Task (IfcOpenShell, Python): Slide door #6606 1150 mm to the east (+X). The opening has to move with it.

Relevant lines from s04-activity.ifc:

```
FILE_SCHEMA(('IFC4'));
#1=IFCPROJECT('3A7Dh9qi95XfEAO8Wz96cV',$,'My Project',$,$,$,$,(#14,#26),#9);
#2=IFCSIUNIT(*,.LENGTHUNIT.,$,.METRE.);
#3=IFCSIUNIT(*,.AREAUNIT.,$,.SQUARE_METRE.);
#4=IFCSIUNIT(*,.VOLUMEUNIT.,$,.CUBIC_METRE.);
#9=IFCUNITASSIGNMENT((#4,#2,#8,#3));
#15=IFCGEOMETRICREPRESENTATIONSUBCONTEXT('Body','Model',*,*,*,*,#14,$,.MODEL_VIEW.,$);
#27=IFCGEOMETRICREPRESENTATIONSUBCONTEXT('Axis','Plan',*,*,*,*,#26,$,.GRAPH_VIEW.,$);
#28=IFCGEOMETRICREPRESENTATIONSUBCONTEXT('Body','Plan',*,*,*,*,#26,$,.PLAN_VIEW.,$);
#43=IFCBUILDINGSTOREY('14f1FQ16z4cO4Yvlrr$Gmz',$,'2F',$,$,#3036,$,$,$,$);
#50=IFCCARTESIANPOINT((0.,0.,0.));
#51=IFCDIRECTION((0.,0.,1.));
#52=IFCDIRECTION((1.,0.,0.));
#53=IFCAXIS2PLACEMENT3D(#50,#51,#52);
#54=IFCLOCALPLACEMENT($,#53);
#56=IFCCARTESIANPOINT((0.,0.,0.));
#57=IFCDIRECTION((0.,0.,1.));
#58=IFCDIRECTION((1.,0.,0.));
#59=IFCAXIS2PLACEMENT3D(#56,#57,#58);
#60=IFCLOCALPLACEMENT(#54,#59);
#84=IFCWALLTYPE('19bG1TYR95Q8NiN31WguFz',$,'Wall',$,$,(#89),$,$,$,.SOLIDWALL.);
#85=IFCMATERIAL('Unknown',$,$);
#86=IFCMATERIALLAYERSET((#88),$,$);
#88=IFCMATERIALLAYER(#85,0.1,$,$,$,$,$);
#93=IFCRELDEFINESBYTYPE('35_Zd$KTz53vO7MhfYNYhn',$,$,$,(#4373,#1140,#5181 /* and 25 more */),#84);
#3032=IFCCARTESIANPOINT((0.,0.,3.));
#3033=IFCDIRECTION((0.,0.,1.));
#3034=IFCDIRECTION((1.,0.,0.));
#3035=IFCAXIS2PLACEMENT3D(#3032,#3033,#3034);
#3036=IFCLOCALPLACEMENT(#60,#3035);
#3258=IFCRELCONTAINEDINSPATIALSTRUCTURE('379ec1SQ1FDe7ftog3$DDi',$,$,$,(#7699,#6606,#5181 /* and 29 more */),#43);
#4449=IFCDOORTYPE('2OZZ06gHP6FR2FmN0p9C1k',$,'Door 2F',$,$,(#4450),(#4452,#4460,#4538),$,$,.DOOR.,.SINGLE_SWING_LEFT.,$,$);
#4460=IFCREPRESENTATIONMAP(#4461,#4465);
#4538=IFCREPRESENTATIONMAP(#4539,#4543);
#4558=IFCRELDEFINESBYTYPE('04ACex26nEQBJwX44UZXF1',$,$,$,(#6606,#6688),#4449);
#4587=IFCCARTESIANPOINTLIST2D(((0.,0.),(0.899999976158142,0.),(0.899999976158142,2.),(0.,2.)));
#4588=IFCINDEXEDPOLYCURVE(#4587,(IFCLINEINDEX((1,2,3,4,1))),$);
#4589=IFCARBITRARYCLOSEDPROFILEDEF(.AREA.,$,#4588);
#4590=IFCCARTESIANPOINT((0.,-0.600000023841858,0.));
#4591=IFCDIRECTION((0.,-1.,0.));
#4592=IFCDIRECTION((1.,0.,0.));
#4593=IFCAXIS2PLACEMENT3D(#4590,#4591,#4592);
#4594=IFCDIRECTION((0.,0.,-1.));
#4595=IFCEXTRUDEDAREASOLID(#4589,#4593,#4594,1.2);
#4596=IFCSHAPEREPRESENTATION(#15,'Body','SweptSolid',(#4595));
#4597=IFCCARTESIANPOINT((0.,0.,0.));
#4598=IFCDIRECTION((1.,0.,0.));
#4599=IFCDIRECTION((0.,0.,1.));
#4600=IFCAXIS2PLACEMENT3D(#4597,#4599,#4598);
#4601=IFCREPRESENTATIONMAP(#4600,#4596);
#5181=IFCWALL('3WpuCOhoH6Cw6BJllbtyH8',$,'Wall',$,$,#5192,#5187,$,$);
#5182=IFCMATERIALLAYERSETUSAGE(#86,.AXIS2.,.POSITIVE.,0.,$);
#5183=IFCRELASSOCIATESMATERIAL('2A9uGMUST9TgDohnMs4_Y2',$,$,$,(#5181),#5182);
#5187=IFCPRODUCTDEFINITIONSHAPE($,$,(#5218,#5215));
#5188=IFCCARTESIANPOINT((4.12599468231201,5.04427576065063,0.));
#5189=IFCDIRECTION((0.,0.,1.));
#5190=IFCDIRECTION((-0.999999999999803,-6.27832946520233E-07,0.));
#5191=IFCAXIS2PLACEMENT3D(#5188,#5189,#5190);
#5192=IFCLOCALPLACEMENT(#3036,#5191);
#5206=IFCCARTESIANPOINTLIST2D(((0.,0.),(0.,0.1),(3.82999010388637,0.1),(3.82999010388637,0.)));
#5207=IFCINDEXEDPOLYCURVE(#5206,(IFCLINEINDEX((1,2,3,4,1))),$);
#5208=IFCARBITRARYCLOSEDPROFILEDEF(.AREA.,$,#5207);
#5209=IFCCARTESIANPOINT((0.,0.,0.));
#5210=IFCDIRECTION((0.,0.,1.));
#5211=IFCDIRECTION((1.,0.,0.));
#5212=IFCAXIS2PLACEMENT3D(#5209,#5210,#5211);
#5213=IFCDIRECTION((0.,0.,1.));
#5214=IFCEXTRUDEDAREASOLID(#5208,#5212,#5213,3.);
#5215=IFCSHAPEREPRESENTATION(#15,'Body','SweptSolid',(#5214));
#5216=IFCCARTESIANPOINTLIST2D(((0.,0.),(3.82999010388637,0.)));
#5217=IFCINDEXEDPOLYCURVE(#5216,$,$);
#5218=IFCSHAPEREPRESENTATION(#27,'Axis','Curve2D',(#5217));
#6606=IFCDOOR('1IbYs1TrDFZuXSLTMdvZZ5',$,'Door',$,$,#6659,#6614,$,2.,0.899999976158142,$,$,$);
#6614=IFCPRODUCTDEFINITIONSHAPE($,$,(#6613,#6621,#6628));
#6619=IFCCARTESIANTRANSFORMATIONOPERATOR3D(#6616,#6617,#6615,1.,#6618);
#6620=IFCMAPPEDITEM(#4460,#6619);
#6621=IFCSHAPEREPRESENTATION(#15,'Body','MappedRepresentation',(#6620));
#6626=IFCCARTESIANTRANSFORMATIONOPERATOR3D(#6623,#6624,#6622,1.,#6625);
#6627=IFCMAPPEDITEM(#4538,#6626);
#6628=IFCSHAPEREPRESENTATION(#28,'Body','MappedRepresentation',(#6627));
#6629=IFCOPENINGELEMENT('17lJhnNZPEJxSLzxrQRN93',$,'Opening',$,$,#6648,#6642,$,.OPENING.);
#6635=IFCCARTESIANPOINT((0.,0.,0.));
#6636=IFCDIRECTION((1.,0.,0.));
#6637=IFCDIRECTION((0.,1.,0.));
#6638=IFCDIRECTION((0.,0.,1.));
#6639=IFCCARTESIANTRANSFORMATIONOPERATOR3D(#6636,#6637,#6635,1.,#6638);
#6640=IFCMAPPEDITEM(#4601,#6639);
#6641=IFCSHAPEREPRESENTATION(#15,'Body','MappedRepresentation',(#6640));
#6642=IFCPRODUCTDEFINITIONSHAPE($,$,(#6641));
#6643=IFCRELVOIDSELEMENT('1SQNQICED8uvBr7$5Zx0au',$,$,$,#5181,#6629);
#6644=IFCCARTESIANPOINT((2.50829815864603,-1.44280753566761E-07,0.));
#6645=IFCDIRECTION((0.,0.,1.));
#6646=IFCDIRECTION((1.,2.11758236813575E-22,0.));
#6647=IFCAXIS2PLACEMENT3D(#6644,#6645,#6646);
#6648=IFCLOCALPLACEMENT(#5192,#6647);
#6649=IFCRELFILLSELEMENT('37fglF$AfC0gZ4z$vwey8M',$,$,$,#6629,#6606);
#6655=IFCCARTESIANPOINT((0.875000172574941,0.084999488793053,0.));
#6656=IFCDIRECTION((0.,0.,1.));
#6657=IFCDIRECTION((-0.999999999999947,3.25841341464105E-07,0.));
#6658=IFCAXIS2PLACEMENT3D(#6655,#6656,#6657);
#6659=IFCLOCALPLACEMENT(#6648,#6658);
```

```python
import ifcopenshell
import ifcopenshell.api.geometry
import ifcopenshell.util.placement
import ifcopenshell.util.unit

model = ifcopenshell.open("s04-activity.ifc")
unit_scale = ifcopenshell.util.unit.calculate_unit_scale(model)

door = model.by_id(6606)
opening = door.FillsVoids[0].RelatingOpeningElement
wall = opening.VoidsElements[0].RelatingBuildingElement

wall_matrix = ifcopenshell.util.placement.get_local_placement(wall.ObjectPlacement)
shift = wall_matrix[:3, 0] * -1.15 / unit_scale
before = ifcopenshell.util.placement.get_local_placement(door.ObjectPlacement)[:3, 3].copy()

# The door is placed relative to its opening, so it follows when the opening moves.
matrix = ifcopenshell.util.placement.get_local_placement(opening.ObjectPlacement)
matrix[:3, 3] += shift
ifcopenshell.api.geometry.edit_object_placement(
    model, product=opening, matrix=matrix, is_si=False, should_transform_children=True
)

after = ifcopenshell.util.placement.get_local_placement(door.ObjectPlacement)[:3, 3]
print("door moved by", (after - before).round(3) + 0.0)

model.write("s04-activity-out.ifc")
```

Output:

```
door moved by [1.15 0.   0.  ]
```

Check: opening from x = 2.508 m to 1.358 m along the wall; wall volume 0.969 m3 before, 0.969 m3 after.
